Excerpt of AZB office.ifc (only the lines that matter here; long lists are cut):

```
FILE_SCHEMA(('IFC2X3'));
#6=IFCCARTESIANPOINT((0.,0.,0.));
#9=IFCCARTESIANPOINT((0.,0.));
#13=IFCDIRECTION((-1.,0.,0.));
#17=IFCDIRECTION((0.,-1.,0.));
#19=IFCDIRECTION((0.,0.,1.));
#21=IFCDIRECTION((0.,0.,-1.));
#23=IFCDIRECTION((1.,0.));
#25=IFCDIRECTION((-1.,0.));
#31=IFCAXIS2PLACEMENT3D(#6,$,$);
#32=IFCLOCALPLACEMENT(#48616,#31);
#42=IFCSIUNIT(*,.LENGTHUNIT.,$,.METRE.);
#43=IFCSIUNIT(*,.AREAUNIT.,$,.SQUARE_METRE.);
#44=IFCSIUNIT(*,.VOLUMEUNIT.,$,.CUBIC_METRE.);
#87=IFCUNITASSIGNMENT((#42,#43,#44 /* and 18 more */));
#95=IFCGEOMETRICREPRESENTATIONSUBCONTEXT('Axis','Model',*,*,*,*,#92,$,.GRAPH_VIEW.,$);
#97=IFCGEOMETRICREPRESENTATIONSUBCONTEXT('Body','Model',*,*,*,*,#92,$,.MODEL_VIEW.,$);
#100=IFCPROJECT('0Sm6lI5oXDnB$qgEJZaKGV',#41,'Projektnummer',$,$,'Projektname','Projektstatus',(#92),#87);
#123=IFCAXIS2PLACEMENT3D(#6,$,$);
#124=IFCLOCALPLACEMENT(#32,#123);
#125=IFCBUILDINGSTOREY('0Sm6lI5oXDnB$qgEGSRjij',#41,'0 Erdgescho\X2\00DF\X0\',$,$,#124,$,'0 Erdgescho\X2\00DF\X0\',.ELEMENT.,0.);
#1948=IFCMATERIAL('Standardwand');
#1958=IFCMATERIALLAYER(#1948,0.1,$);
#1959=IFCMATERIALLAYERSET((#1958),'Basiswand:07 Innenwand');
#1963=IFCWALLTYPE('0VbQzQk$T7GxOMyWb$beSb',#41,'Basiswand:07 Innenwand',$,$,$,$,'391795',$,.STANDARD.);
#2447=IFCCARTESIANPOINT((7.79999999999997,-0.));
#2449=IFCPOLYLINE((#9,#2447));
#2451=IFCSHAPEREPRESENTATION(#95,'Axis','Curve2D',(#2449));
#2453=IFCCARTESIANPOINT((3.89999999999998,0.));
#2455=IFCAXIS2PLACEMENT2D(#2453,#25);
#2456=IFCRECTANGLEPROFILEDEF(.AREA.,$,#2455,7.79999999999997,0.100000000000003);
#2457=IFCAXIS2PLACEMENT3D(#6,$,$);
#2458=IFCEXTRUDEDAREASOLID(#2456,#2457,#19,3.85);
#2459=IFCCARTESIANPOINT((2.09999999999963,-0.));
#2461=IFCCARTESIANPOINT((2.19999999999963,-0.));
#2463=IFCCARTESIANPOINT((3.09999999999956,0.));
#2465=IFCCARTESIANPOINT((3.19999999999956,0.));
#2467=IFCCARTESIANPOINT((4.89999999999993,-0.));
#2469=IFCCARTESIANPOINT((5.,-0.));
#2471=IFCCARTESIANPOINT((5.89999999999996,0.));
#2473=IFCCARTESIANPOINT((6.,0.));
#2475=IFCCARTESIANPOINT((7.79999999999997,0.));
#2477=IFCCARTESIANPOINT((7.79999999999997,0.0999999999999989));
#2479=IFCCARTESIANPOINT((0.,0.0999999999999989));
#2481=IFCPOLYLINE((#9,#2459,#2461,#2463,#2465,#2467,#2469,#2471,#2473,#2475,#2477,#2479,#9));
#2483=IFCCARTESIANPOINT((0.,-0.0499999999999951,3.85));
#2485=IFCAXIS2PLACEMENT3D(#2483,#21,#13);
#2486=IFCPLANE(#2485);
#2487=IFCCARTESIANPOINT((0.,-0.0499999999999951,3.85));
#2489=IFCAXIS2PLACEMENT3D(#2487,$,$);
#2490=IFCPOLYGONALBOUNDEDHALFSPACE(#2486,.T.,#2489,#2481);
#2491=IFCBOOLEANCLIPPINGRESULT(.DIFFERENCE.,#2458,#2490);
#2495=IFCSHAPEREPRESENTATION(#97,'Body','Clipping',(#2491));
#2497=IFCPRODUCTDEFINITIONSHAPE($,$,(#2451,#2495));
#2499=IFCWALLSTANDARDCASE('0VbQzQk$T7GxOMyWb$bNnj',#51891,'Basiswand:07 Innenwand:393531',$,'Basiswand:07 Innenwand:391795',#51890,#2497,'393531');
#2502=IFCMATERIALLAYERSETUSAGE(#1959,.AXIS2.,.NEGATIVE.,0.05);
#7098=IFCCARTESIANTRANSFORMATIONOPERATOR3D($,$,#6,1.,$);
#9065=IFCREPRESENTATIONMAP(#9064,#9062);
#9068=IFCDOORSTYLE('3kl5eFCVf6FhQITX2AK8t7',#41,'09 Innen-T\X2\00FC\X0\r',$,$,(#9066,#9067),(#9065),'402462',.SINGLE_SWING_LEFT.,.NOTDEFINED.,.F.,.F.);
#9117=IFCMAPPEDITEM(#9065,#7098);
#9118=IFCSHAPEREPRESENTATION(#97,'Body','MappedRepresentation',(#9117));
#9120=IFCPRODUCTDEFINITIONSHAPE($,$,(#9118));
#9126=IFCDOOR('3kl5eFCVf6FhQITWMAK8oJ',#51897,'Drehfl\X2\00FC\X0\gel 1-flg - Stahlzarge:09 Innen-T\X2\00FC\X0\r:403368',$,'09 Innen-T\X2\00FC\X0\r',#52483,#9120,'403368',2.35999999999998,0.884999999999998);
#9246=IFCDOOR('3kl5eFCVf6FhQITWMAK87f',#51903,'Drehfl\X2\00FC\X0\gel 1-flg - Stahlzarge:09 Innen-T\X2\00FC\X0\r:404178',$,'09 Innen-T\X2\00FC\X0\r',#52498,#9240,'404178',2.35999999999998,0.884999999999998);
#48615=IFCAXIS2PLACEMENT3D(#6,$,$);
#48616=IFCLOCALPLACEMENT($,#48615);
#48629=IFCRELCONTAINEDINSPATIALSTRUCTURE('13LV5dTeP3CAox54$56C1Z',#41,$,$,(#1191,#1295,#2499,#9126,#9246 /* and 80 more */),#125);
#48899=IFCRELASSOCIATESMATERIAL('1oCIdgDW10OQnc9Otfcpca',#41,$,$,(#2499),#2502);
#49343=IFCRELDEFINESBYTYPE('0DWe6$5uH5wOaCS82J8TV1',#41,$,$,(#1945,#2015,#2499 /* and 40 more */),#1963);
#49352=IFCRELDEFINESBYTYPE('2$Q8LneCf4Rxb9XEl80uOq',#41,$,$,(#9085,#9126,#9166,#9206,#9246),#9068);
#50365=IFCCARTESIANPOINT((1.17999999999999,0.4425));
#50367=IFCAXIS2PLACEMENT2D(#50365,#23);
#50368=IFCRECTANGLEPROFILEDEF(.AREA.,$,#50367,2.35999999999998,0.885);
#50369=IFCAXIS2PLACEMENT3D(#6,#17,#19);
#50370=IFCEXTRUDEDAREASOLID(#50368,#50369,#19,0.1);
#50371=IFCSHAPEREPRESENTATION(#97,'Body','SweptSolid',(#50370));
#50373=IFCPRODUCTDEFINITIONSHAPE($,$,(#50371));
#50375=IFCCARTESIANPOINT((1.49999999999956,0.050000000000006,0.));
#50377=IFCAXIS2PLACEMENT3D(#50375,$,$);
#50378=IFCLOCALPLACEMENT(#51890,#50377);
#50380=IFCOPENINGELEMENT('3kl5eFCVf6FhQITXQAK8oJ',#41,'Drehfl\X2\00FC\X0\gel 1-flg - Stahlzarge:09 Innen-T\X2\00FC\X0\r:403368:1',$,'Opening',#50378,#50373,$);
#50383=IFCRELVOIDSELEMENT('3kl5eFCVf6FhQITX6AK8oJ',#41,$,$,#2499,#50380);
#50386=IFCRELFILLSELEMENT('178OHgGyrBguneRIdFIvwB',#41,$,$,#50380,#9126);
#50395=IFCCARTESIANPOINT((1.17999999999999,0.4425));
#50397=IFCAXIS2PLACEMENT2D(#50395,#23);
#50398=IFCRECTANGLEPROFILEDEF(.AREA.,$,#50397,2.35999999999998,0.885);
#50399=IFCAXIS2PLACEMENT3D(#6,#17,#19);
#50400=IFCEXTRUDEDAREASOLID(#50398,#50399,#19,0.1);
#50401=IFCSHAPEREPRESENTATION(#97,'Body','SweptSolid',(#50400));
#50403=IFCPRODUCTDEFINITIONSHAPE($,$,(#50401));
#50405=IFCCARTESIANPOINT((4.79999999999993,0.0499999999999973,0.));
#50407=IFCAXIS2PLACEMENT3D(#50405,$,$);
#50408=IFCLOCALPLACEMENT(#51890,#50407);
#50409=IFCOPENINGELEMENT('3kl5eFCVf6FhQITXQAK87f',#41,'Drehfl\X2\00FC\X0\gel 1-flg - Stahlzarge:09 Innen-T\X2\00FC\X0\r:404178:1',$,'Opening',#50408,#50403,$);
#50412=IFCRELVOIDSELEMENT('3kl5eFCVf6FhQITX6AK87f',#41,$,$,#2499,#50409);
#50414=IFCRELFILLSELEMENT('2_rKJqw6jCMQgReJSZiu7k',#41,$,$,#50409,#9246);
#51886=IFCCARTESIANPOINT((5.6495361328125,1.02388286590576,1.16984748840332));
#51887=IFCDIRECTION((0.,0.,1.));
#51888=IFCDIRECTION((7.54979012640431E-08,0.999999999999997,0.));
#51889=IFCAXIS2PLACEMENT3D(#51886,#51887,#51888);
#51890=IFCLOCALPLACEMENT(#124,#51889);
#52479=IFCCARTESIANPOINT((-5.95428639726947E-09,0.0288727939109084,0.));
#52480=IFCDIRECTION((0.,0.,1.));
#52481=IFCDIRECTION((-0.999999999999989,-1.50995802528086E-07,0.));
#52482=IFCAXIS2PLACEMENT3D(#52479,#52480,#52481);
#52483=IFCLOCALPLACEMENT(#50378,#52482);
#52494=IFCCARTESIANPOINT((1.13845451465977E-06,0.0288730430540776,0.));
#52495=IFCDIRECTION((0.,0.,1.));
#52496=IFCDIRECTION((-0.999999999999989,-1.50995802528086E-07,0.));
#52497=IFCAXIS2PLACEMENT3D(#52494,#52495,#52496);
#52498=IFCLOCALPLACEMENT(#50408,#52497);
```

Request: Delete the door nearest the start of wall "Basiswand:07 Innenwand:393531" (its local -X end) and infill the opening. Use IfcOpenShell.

```python
import ifcopenshell
import ifcopenshell.api.feature
import ifcopenshell.api.root
import ifcopenshell.geom
import ifcopenshell.util.shape

model = ifcopenshell.open("AZB office.ifc")
settings = ifcopenshell.geom.settings()


def volume(element):
    """Net volume in cubic metres, openings subtracted."""
    shape = ifcopenshell.geom.create_shape(settings, element)
    return ifcopenshell.util.shape.get_volume(shape.geometry)


door = model.by_id(9126)
opening = door.FillsVoids[0].RelatingOpeningElement
wall = opening.VoidsElements[0].RelatingBuildingElement
before = volume(wall)

ifcopenshell.api.root.remove_product(model, product=door)
ifcopenshell.api.feature.remove_feature(model, feature=opening)

after = volume(wall)

print(f"wall volume {before:.3f} -> {after:.3f} m3")

model.write("AZB office_updated.ifc")
```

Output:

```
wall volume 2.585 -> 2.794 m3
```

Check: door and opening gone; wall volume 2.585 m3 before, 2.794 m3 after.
